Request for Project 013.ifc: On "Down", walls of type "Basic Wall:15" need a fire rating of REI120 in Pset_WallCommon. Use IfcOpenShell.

First a look at what the model holds.

```python
import ifcopenshell
import ifcopenshell.util.element

model = ifcopenshell.open("Project 013.ifc")
print(model.schema)
storey = next(s for s in model.by_type("IfcBuildingStorey") if s.Name == "Down")
walls = [e for e in ifcopenshell.util.element.get_decomposition(storey) if e.is_a("IfcWall")]
seen = {}
for e in walls:
    element_type = ifcopenshell.util.element.get_type(e)
    key = (element_type.Name if element_type != e and element_type else None, ifcopenshell.util.element.get_pset(e, "Pset_WallCommon", "FireRating"))
    seen[key] = seen.get(key, 0) + 1
for (name, value), count in sorted(seen.items(), key=str):
    print(count, "x", name, "|", value)
```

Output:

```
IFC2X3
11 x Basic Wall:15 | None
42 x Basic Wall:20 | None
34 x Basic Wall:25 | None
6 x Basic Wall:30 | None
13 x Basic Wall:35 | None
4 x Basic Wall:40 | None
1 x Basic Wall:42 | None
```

```python
import ifcopenshell
import ifcopenshell.api.pset
import ifcopenshell.util.element

model = ifcopenshell.open("Project 013.ifc")

storey = next(s for s in model.by_type("IfcBuildingStorey") if s.Name == "Down")
walls = [e for e in ifcopenshell.util.element.get_decomposition(storey) if e.is_a("IfcWall")]

count = 0
for e in walls:
    element_type = ifcopenshell.util.element.get_type(e)
    if element_type in (None, e) or element_type.Name != "Basic Wall:15":
        continue
    # add_pset returns the element's existing set when there is one.
    pset = ifcopenshell.api.pset.add_pset(model, product=e, name="Pset_WallCommon")
    ifcopenshell.api.pset.edit_pset(model, pset=pset, properties={"FireRating": "REI120"})
    count += 1

print(count, "walls updated")

model.write("Project 013_updated.ifc")
```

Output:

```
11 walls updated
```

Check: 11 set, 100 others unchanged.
